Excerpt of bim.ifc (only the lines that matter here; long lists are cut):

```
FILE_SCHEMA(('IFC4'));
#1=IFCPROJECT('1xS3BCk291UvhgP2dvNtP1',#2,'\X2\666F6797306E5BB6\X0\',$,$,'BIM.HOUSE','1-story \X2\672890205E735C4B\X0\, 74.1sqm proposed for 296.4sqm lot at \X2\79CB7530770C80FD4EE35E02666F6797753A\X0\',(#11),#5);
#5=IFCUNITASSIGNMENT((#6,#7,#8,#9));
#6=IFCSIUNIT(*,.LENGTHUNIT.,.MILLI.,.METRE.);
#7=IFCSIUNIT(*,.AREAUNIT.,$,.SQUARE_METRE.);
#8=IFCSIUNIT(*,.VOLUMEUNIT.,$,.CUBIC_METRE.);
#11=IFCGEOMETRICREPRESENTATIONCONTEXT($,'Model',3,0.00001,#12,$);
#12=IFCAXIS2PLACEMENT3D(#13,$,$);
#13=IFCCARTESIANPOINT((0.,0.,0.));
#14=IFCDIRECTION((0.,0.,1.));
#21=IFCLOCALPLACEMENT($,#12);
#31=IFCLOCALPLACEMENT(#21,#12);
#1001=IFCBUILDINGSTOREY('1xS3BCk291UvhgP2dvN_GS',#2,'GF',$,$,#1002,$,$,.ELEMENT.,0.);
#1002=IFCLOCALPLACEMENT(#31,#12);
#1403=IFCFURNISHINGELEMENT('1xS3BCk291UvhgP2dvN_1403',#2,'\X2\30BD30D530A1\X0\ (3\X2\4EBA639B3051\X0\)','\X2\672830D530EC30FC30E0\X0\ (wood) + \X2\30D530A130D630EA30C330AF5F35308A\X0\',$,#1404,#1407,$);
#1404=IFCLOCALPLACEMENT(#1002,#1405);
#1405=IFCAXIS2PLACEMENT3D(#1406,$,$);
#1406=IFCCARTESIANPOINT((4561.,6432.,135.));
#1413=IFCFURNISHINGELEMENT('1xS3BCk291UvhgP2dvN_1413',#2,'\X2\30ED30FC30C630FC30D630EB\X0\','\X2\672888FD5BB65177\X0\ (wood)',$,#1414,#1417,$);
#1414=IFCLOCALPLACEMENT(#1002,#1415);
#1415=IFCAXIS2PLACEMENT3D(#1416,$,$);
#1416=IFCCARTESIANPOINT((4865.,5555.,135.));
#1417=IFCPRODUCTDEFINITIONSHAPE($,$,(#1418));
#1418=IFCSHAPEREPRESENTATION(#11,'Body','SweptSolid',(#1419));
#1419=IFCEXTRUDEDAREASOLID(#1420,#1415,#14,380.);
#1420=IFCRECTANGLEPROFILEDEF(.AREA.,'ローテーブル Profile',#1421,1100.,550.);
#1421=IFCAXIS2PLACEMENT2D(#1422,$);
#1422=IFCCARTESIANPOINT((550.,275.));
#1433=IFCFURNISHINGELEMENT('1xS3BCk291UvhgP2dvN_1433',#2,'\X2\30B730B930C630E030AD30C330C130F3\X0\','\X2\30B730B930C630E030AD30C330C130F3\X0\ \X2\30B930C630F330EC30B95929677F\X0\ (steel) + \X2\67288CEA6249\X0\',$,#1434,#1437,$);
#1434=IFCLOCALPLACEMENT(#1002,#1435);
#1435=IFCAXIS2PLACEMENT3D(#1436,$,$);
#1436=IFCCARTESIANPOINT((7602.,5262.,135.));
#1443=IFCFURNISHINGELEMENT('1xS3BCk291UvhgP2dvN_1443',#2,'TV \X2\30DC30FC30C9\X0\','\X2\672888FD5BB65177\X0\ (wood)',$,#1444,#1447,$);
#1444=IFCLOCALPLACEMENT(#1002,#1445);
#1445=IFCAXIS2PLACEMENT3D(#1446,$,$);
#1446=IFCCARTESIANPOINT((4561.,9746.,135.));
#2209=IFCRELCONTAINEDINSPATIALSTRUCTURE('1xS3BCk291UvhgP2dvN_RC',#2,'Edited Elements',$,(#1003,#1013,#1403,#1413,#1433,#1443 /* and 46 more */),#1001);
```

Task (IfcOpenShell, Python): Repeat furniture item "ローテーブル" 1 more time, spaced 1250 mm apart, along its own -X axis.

```python
import ifcopenshell
import ifcopenshell.api.geometry
import ifcopenshell.api.root
import ifcopenshell.util.element
import ifcopenshell.util.placement

model = ifcopenshell.open("bim.ifc")


def reuse_history(source, copy):
    """copy_class also copies each property set's owner history, people and application; keep the originals."""
    for rel in copy.IsDefinedBy:
        if rel.is_a("IfcRelDefinesByProperties") and (history := rel.RelatingPropertyDefinition.OwnerHistory):
            rel.RelatingPropertyDefinition.OwnerHistory = source.OwnerHistory
            ifcopenshell.util.element.remove_deep2(model, history)


source = model.by_guid("1xS3BCk291UvhgP2dvN_1413")
base = ifcopenshell.util.placement.get_local_placement(source.ObjectPlacement)
step = -base[:3, 0] * 1250.0

for i in range(1, 2):
    copy = ifcopenshell.api.root.copy_class(model, product=source)
    copy.Representation = ifcopenshell.util.element.copy_deep(
        model, source.Representation, exclude=["IfcGeometricRepresentationContext", "IfcRepresentationMap"]
    )
    reuse_history(source, copy)
    matrix = base.copy()
    matrix[:3, 3] += i * step
    print("added at", matrix[:3, 3].round(3) + 0.0)
    ifcopenshell.api.geometry.edit_object_placement(model, product=copy, matrix=matrix, is_si=False)

model.write("bim-out.ifc")
```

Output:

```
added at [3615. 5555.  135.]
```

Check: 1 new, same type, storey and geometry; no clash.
